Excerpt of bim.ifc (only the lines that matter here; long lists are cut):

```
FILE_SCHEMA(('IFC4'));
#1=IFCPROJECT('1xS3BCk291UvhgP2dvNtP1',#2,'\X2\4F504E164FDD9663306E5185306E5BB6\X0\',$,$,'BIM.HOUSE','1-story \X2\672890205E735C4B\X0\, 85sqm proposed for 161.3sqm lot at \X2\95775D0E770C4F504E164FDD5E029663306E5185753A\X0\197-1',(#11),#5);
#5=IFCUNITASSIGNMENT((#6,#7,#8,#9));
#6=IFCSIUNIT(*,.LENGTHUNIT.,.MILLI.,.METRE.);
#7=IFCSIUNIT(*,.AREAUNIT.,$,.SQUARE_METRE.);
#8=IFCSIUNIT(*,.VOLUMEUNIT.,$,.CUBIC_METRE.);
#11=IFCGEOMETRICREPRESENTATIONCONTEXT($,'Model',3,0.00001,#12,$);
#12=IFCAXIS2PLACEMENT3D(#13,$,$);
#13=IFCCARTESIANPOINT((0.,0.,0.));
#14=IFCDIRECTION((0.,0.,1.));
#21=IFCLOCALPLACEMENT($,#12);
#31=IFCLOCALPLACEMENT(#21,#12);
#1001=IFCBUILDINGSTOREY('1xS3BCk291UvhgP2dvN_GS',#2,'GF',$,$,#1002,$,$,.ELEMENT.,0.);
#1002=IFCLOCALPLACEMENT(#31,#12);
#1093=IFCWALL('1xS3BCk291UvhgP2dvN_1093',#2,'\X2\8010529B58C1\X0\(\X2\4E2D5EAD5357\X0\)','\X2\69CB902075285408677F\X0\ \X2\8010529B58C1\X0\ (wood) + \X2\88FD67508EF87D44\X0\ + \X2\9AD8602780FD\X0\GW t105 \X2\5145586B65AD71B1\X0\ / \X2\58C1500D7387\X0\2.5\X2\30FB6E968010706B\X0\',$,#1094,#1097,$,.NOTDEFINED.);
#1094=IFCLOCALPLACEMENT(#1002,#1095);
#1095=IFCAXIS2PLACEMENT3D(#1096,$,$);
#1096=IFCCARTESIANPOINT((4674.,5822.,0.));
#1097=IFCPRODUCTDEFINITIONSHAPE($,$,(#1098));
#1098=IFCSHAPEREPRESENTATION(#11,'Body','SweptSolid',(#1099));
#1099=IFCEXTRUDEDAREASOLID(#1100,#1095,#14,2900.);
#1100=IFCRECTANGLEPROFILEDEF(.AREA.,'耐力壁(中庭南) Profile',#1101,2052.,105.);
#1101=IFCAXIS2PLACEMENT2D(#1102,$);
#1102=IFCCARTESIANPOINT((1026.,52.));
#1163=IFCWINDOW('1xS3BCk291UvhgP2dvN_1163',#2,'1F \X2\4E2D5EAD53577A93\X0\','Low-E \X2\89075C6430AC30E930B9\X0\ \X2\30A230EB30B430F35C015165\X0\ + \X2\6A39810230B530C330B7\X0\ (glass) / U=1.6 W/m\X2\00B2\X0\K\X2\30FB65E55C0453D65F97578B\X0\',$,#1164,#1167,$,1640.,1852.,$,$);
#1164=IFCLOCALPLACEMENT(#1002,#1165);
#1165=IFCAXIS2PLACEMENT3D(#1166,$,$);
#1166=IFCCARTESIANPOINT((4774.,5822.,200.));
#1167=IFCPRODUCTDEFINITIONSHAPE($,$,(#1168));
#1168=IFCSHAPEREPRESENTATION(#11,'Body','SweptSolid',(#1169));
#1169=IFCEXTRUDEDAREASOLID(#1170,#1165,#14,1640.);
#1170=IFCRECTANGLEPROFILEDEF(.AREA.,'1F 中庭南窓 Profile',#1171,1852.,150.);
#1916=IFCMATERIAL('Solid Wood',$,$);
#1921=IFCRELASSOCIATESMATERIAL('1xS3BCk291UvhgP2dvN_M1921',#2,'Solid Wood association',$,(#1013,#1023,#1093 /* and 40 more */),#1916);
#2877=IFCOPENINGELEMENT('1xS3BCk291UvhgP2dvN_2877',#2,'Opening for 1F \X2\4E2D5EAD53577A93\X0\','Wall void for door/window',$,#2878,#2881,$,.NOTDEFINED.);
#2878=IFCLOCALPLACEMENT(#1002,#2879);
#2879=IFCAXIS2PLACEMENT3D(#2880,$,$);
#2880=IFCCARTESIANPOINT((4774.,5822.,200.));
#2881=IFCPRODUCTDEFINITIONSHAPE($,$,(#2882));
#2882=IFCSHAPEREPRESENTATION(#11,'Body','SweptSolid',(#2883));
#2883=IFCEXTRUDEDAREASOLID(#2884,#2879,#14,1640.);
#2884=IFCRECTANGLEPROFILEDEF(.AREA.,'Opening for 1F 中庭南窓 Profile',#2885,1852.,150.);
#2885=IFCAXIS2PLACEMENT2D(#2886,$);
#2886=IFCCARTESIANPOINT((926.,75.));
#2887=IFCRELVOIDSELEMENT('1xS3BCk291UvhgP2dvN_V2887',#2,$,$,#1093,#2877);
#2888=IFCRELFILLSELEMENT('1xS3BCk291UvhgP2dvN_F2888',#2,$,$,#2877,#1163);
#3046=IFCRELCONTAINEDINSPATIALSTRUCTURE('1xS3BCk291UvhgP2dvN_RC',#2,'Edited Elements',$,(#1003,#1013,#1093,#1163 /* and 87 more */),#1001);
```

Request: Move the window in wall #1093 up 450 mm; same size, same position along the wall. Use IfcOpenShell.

```python
import numpy as np
import ifcopenshell
import ifcopenshell.api.geometry
import ifcopenshell.util.placement
import ifcopenshell.util.unit

model = ifcopenshell.open("bim.ifc")
unit_scale = ifcopenshell.util.unit.calculate_unit_scale(model)

window = model.by_guid("1xS3BCk291UvhgP2dvN_1163")
opening = window.FillsVoids[0].RelatingOpeningElement
dz = 0.45 / unit_scale

shift = np.array([0.0, 0.0, dz])
# The window is not placed relative to its opening, so move both.
for product in (opening, window):
    matrix = ifcopenshell.util.placement.get_local_placement(product.ObjectPlacement)
    matrix[:3, 3] += shift
    ifcopenshell.api.geometry.edit_object_placement(model, product=product, matrix=matrix, is_si=False)

print(f"moved by {dz * unit_scale:+.3f} m")

model.write("bim_updated.ifc")
```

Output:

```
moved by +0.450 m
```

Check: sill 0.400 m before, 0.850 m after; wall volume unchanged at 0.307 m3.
